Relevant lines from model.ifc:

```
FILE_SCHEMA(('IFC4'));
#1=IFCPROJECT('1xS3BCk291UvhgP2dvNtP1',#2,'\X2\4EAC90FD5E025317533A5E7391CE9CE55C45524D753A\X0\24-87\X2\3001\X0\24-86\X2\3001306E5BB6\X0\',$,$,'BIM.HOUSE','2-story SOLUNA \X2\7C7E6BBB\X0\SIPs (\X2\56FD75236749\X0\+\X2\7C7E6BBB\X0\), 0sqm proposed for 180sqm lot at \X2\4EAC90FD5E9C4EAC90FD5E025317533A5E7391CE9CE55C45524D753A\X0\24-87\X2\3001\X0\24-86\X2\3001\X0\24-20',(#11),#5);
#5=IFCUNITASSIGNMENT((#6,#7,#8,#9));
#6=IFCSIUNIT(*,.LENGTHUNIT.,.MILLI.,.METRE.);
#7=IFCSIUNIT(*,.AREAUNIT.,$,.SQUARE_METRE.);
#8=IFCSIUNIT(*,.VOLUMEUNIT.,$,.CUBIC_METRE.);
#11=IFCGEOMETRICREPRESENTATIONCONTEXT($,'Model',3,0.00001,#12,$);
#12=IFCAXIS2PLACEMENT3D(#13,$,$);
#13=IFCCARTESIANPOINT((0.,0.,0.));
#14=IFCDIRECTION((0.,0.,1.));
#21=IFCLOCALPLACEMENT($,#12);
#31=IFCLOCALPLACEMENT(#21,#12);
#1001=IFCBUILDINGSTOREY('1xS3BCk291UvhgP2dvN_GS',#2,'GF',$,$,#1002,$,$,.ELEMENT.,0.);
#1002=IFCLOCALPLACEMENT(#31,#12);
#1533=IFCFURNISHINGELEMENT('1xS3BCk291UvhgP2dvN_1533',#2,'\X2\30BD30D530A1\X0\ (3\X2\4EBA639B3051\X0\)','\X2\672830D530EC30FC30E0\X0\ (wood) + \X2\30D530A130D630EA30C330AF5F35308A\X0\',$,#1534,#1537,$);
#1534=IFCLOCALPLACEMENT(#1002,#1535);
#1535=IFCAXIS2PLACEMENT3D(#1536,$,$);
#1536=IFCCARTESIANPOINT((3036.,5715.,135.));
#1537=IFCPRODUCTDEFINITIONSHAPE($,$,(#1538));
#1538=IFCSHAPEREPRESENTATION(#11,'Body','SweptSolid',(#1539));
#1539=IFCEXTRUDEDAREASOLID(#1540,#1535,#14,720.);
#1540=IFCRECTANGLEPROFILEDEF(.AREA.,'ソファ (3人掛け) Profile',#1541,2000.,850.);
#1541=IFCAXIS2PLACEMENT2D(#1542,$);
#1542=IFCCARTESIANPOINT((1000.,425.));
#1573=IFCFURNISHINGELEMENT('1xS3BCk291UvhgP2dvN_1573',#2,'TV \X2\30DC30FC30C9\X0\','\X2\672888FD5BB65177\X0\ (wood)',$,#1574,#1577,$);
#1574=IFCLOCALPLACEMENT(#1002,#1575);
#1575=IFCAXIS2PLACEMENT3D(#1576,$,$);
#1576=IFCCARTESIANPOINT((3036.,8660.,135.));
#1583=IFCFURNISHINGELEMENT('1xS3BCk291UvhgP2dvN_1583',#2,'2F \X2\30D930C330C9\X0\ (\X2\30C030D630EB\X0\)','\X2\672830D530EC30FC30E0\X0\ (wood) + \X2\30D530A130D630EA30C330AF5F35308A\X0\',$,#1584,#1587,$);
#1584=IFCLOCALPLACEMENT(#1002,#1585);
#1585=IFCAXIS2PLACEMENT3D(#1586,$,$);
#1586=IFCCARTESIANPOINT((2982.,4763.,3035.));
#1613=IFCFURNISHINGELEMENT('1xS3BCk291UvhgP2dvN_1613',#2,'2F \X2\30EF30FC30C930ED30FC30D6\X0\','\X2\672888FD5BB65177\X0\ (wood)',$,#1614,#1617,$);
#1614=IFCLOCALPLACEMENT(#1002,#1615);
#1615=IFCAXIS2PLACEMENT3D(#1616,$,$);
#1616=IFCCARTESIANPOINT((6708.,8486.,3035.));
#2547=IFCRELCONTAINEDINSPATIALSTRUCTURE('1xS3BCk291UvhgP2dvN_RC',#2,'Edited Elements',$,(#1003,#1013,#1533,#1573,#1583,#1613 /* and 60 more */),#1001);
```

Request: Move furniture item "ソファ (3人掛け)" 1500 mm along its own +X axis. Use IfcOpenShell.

```python
import ifcopenshell
import ifcopenshell.api.geometry
import ifcopenshell.util.placement

model = ifcopenshell.open("model.ifc")

item = model.by_id(1533)
matrix = ifcopenshell.util.placement.get_local_placement(item.ObjectPlacement)
matrix[:3, 3] += matrix[:3, 0] * 1500.0
ifcopenshell.api.geometry.edit_object_placement(model, product=item, matrix=matrix, is_si=False)

print(ifcopenshell.util.placement.get_local_placement(item.ObjectPlacement).round(3) + 0.0)

model.write("model_edited.ifc")
```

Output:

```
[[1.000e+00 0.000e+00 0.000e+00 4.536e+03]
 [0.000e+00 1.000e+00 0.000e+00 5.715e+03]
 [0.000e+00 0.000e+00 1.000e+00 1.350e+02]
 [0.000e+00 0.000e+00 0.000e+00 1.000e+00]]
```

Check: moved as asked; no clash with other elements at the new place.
